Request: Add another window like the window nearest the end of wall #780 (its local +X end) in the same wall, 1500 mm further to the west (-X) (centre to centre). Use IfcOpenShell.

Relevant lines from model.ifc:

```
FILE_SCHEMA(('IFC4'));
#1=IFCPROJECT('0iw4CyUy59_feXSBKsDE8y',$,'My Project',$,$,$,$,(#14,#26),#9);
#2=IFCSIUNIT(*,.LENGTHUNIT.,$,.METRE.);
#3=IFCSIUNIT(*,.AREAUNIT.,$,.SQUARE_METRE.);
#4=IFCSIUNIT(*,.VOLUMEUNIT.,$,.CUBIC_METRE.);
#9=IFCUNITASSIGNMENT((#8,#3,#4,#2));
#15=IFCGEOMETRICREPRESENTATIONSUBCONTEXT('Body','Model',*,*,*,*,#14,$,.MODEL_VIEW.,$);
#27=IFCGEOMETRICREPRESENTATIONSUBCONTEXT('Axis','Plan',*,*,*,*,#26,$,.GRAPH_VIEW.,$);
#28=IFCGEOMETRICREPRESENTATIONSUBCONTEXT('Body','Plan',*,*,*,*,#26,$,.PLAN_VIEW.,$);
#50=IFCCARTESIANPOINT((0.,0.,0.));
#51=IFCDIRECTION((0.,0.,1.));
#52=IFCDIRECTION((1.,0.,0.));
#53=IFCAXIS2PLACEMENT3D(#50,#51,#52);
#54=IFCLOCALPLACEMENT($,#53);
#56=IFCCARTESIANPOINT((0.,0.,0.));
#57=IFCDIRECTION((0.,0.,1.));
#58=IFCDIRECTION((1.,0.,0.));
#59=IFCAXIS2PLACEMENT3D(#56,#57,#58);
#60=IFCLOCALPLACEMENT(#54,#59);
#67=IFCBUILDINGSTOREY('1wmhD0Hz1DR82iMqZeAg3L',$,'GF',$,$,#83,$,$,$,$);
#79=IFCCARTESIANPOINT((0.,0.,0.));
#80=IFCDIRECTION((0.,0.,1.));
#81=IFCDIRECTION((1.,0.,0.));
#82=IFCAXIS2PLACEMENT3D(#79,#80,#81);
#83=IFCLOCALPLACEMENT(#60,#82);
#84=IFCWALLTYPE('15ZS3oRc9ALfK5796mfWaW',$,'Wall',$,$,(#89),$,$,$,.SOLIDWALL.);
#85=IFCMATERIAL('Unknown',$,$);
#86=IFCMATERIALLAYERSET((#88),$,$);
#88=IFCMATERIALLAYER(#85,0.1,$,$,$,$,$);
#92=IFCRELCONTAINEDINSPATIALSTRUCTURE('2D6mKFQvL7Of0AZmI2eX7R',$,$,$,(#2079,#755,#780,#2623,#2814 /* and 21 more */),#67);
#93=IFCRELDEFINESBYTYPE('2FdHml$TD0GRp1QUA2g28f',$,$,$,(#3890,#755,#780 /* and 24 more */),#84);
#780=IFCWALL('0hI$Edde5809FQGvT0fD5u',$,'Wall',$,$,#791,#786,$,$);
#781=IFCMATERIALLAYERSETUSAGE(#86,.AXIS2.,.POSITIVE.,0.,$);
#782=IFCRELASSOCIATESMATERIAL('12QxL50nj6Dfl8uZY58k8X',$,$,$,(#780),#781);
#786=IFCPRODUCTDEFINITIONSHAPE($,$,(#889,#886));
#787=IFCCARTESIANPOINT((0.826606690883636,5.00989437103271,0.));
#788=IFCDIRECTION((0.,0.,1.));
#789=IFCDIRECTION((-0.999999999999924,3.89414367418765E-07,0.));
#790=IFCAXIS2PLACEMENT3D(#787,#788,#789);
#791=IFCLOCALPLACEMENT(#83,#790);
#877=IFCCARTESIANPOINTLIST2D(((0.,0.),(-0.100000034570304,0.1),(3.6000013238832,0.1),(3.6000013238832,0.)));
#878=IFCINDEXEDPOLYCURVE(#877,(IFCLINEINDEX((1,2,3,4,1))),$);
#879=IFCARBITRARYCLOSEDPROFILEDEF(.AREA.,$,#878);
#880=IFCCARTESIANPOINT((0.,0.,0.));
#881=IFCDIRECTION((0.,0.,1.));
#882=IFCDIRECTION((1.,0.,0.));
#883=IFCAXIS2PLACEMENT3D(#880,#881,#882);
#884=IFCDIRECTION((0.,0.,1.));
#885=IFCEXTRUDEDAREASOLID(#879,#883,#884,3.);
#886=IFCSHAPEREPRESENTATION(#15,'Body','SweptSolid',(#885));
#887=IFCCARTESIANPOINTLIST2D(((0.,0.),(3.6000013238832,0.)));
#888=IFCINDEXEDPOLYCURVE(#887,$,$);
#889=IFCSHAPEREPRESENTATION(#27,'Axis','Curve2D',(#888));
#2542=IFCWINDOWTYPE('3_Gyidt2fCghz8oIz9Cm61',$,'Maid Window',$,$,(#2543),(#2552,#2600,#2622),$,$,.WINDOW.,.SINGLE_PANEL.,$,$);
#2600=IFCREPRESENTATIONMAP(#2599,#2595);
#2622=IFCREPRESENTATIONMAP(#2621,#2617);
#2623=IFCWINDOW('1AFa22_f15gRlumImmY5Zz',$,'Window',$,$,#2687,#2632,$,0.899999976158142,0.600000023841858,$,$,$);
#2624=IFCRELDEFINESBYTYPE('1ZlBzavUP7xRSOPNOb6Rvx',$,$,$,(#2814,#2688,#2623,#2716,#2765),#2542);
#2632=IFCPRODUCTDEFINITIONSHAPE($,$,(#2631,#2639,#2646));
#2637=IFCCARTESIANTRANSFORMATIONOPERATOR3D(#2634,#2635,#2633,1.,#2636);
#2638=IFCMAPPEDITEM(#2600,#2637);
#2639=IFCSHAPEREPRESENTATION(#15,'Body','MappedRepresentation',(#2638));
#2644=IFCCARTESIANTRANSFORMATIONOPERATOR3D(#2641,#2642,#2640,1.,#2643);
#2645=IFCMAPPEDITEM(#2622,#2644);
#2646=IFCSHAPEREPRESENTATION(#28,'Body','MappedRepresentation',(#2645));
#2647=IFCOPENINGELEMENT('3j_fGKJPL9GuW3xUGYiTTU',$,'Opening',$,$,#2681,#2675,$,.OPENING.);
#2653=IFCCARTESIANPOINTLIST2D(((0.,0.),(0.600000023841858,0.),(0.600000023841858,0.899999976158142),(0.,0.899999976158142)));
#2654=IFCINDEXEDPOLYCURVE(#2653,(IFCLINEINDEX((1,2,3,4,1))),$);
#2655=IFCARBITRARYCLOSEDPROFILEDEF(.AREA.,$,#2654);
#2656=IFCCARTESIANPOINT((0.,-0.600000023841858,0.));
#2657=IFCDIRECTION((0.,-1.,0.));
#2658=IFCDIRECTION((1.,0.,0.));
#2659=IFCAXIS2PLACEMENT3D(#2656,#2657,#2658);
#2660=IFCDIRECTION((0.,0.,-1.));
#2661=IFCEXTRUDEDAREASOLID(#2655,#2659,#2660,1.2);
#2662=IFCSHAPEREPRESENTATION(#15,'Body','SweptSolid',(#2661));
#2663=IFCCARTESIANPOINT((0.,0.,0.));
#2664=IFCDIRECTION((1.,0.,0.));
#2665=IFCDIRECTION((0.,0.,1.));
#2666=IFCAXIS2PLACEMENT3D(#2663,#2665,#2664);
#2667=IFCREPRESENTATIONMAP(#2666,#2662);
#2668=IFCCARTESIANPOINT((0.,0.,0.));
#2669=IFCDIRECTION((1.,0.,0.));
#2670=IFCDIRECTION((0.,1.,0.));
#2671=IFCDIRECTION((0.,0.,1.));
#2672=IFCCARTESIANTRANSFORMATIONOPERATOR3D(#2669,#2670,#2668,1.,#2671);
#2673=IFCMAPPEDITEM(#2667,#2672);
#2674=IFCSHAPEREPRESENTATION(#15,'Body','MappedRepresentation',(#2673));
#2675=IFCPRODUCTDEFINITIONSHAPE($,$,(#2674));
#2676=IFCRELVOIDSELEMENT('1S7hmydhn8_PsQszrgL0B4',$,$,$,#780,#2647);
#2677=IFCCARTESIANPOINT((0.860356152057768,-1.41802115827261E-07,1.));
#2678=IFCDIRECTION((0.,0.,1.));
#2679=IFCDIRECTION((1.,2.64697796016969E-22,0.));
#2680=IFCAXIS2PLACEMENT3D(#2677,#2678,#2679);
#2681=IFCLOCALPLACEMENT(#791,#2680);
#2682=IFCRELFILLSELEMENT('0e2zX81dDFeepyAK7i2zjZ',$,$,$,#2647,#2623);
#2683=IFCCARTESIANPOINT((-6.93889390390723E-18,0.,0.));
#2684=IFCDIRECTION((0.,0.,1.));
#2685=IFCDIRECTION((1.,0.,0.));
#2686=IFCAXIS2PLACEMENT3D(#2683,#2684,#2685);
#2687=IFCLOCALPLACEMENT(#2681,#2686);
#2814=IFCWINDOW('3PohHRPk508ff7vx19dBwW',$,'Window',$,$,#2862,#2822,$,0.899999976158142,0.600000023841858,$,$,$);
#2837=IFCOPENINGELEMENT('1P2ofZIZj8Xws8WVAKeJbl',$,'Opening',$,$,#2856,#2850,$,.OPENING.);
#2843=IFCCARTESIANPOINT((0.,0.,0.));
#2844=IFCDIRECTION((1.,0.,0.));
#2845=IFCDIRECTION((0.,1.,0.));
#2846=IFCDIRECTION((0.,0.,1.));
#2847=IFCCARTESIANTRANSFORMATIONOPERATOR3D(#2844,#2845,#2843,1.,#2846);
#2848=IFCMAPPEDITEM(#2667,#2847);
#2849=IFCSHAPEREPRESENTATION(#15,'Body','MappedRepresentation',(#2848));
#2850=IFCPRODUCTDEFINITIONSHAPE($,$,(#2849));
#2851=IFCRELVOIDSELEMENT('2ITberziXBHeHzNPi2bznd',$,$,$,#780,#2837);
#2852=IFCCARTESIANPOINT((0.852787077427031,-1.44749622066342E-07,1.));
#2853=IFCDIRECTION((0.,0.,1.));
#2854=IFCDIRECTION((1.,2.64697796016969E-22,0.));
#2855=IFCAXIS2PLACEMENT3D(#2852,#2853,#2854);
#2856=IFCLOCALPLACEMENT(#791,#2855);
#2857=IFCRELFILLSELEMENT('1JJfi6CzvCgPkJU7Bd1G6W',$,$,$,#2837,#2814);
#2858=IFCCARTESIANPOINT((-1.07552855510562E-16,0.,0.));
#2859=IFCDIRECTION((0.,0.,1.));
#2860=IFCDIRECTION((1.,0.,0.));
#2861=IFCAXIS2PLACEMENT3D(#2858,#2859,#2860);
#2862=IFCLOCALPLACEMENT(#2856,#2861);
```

```python
import ifcopenshell
import ifcopenshell.api.feature
import ifcopenshell.api.geometry
import ifcopenshell.api.root
import ifcopenshell.geom
import ifcopenshell.util.element
import ifcopenshell.util.placement
import ifcopenshell.util.shape

model = ifcopenshell.open("model.ifc")
settings = ifcopenshell.geom.settings()


def volume(element):
    """Net volume in cubic metres, openings subtracted."""
    shape = ifcopenshell.geom.create_shape(settings, element)
    return ifcopenshell.util.shape.get_volume(shape.geometry)


window = model.by_guid("1AFa22_f15gRlumImmY5Zz")
opening = window.FillsVoids[0].RelatingOpeningElement
wall = opening.VoidsElements[0].RelatingBuildingElement
before = volume(wall)
shift = ifcopenshell.util.placement.get_local_placement(wall.ObjectPlacement)[:3, 0] * 1.5

# copy_class copies the void relationship, type, container and properties, but no geometry.
new_opening = ifcopenshell.api.root.copy_class(model, product=opening)
new_opening.Representation = ifcopenshell.util.element.copy_deep(
    model, opening.Representation, exclude=["IfcGeometricRepresentationContext", "IfcRepresentationMap"]
)
new_window = ifcopenshell.api.root.copy_class(model, product=window)
new_window.Representation = ifcopenshell.util.element.copy_deep(
    model, window.Representation, exclude=["IfcGeometricRepresentationContext", "IfcRepresentationMap"]
)
ifcopenshell.api.feature.add_filling(model, opening=new_opening, element=new_window)

for old, new in ((opening, new_opening), (window, new_window)):
    matrix = ifcopenshell.util.placement.get_local_placement(old.ObjectPlacement)
    matrix[:3, 3] += shift
    ifcopenshell.api.geometry.edit_object_placement(model, product=new, matrix=matrix, is_si=False)

after = volume(wall)

print(f"wall volume {before:.3f} -> {after:.3f} m3")

model.write("model_v2.ifc")
```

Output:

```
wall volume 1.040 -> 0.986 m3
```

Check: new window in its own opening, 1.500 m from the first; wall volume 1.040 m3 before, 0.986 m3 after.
